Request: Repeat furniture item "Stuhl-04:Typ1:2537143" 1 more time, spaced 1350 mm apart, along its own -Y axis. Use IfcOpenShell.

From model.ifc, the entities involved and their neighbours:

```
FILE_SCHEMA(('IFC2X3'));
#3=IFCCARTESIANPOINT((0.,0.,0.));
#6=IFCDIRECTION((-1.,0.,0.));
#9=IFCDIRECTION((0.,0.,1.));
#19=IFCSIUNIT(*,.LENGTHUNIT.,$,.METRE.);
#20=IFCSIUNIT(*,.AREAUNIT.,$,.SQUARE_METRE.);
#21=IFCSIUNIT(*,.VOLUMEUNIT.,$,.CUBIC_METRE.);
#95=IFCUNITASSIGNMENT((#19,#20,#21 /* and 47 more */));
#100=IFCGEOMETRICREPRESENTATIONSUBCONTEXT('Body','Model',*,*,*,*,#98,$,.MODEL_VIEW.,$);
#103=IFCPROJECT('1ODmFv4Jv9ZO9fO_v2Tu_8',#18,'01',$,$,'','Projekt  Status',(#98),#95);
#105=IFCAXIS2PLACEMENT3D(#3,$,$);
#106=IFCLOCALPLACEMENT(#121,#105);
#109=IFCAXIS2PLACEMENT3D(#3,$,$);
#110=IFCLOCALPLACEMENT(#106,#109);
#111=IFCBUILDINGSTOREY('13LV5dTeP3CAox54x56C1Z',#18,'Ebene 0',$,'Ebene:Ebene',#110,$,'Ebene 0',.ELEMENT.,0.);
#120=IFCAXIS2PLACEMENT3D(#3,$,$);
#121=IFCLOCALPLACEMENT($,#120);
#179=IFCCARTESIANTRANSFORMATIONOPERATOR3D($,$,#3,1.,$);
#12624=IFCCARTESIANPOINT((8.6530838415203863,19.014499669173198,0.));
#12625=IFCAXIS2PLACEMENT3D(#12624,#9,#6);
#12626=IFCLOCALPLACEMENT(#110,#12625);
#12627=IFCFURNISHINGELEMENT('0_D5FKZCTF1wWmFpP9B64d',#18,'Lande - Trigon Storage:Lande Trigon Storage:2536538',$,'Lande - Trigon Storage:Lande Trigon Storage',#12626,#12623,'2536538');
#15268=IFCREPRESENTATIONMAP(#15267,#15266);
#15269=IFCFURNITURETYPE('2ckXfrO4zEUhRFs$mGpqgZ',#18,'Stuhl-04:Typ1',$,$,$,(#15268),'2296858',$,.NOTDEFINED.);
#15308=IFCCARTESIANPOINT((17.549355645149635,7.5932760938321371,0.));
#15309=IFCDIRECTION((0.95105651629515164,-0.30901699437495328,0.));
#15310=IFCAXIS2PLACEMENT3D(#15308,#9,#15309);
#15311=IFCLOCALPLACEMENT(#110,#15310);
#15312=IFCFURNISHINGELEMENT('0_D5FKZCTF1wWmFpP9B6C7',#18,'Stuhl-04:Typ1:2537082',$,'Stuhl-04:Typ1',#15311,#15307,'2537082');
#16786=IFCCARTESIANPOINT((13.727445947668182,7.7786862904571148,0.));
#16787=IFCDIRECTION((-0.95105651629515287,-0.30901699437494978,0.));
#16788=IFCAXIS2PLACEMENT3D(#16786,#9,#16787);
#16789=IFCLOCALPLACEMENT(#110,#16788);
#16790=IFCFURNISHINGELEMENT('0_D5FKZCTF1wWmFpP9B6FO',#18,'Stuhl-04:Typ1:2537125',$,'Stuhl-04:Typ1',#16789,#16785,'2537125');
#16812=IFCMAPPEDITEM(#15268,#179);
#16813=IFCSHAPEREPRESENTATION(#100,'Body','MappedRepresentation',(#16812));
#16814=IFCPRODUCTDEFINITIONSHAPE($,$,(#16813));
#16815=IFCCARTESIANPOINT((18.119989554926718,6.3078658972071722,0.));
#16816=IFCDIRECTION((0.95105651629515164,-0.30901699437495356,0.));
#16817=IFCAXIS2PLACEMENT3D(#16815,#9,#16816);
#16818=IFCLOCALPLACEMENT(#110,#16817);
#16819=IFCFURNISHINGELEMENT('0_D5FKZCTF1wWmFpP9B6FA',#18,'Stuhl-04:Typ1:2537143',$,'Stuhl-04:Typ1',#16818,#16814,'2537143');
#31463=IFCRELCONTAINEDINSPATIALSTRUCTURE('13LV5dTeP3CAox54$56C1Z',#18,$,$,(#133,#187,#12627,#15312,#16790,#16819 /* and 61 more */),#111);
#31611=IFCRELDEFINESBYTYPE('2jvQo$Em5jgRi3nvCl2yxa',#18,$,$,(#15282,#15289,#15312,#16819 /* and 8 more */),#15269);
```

```python
import ifcopenshell
import ifcopenshell.api.geometry
import ifcopenshell.api.root
import ifcopenshell.util.element
import ifcopenshell.util.placement

model = ifcopenshell.open("model.ifc")

source = model.by_guid("0_D5FKZCTF1wWmFpP9B6FA")
base = ifcopenshell.util.placement.get_local_placement(source.ObjectPlacement)
step = -base[:3, 1] * 1.35

for i in range(1, 2):
    copy = ifcopenshell.api.root.copy_class(model, product=source)
    copy.Representation = ifcopenshell.util.element.copy_deep(
        model, source.Representation, exclude=["IfcGeometricRepresentationContext", "IfcRepresentationMap"]
    )
    copy.Name = "Stuhl-04:Typ1"
    copy.Tag = None
    matrix = base.copy()
    matrix[:3, 3] += i * step
    print("added at", matrix[:3, 3].round(3) + 0.0)
    ifcopenshell.api.geometry.edit_object_placement(model, product=copy, matrix=matrix, is_si=False)

model.write("model_rev.ifc")
```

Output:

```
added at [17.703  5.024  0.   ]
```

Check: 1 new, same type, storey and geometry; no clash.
